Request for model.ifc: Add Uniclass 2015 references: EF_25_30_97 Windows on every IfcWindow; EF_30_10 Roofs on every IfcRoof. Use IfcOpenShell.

First a look at what the model holds.

```python
import ifcopenshell

model = ifcopenshell.open("model.ifc")
print(model.schema)
print("classifications:", [c.Name for c in model.by_type("IfcClassification")])
for ifc_class in ("IfcDoor", "IfcRoof", "IfcStair", "IfcWall", "IfcWindow"):
    print(ifc_class, len(model.by_type(ifc_class)))
```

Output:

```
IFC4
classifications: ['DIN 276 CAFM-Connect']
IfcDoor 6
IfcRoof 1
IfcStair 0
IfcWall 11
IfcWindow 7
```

```python
import ifcopenshell
import ifcopenshell.api.classification

model = ifcopenshell.open("model.ifc")

system = ifcopenshell.api.classification.add_classification(model, classification="Uniclass 2015")

codes = {
    "IfcWindow": ("EF_25_30_97", "Windows"),
    "IfcRoof": ("EF_30_10", "Roofs"),
}
for ifc_class, (code, name) in codes.items():
    products = model.by_type(ifc_class)
    ifcopenshell.api.classification.add_reference(
        model, products=products, classification=system, identification=code, name=name
    )
    print(code, len(products))

model.write("model_edited.ifc")
```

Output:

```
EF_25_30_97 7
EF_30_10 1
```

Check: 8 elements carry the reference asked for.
